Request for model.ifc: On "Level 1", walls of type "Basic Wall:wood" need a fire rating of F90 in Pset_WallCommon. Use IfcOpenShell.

First a look at what the model holds.

```python
import ifcopenshell
import ifcopenshell.util.element

model = ifcopenshell.open("model.ifc")
print(model.schema)
storey = next(s for s in model.by_type("IfcBuildingStorey") if s.Name == "Level 1")
walls = [e for e in ifcopenshell.util.element.get_decomposition(storey) if e.is_a("IfcWall")]
seen = {}
for e in walls:
    element_type = ifcopenshell.util.element.get_type(e)
    key = (element_type.Name if element_type != e and element_type else None, ifcopenshell.util.element.get_pset(e, "Pset_WallCommon", "FireRating"))
    seen[key] = seen.get(key, 0) + 1
for (name, value), count in sorted(seen.items(), key=str):
    print(count, "x", name, "|", value)
```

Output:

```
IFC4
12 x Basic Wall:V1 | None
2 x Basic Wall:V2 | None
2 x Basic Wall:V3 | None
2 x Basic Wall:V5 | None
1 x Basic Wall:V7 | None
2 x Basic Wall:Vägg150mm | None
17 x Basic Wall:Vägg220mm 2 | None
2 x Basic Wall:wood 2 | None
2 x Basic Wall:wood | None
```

```python
import ifcopenshell
import ifcopenshell.api.pset
import ifcopenshell.util.element

model = ifcopenshell.open("model.ifc")

storey = next(s for s in model.by_type("IfcBuildingStorey") if s.Name == "Level 1")
walls = [e for e in ifcopenshell.util.element.get_decomposition(storey) if e.is_a("IfcWall")]

count = 0
for e in walls:
    element_type = ifcopenshell.util.element.get_type(e)
    if element_type in (None, e) or element_type.Name != "Basic Wall:wood":
        continue
    # add_pset returns the element's existing set when there is one.
    pset = ifcopenshell.api.pset.add_pset(model, product=e, name="Pset_WallCommon")
    ifcopenshell.api.pset.edit_pset(model, pset=pset, properties={"FireRating": "F90"})
    count += 1

print(count, "walls updated")

model.write("model_edited.ifc")
```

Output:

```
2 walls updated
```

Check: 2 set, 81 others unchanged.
